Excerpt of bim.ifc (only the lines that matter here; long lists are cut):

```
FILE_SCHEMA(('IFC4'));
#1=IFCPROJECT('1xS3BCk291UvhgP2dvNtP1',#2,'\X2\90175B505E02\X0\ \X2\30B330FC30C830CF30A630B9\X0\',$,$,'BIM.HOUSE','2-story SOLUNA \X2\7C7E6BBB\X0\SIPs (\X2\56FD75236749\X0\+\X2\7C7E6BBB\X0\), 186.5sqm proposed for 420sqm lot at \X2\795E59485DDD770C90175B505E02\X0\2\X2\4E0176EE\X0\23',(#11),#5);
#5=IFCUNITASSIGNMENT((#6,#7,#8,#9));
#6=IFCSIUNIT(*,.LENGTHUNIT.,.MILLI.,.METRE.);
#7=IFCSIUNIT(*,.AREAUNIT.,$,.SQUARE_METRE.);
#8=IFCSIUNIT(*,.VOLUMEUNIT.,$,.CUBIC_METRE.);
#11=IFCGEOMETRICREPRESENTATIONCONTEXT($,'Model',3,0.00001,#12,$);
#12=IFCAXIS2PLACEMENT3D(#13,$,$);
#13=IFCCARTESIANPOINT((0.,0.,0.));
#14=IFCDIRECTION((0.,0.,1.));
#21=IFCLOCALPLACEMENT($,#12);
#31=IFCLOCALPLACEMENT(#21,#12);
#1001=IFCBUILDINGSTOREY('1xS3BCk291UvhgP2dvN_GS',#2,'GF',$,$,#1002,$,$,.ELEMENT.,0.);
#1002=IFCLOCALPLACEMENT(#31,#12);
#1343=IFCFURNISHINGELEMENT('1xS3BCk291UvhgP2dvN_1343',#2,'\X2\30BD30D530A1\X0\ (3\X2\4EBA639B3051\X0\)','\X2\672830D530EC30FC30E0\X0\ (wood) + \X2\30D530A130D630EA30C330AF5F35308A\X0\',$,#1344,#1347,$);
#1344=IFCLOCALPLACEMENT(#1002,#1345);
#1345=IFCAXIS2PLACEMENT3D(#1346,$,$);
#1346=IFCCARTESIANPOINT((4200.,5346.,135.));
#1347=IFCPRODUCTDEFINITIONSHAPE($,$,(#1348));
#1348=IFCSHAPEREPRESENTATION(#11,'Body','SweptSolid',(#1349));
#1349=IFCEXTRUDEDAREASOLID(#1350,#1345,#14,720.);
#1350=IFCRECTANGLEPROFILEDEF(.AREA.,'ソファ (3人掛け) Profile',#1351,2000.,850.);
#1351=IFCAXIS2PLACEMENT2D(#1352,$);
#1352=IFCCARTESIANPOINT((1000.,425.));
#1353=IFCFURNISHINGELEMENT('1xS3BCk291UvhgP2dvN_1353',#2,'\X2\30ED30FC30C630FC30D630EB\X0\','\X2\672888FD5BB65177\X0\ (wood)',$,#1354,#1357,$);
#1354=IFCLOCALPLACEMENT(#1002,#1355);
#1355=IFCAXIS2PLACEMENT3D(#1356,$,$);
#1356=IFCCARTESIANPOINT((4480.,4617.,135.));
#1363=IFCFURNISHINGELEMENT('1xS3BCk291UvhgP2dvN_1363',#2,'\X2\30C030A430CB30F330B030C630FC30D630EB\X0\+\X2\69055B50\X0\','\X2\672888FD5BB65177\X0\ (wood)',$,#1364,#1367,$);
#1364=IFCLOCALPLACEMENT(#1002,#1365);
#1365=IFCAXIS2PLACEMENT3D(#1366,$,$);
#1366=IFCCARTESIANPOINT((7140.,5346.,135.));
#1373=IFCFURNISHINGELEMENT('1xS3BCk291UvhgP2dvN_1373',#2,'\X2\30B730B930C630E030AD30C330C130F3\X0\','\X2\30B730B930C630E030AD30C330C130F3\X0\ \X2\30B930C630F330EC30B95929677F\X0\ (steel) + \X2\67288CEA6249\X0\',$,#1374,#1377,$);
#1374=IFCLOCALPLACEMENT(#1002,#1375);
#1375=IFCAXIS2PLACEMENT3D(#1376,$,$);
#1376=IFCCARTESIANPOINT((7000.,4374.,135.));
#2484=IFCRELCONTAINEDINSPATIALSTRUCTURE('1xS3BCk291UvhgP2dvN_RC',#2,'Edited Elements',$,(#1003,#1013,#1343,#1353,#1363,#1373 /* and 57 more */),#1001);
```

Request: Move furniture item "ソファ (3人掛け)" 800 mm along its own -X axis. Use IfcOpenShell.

```python
import ifcopenshell
import ifcopenshell.api.geometry
import ifcopenshell.util.placement

model = ifcopenshell.open("bim.ifc")

item = model.by_guid("1xS3BCk291UvhgP2dvN_1343")
matrix = ifcopenshell.util.placement.get_local_placement(item.ObjectPlacement)
matrix[:3, 3] -= matrix[:3, 0] * 800.0
ifcopenshell.api.geometry.edit_object_placement(model, product=item, matrix=matrix, is_si=False)

print(ifcopenshell.util.placement.get_local_placement(item.ObjectPlacement).round(3) + 0.0)

model.write("bim_updated.ifc")
```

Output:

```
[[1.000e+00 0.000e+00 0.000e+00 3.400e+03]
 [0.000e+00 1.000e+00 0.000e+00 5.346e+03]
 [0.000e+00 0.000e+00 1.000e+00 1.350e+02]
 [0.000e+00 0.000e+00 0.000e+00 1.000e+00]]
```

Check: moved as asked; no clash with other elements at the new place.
